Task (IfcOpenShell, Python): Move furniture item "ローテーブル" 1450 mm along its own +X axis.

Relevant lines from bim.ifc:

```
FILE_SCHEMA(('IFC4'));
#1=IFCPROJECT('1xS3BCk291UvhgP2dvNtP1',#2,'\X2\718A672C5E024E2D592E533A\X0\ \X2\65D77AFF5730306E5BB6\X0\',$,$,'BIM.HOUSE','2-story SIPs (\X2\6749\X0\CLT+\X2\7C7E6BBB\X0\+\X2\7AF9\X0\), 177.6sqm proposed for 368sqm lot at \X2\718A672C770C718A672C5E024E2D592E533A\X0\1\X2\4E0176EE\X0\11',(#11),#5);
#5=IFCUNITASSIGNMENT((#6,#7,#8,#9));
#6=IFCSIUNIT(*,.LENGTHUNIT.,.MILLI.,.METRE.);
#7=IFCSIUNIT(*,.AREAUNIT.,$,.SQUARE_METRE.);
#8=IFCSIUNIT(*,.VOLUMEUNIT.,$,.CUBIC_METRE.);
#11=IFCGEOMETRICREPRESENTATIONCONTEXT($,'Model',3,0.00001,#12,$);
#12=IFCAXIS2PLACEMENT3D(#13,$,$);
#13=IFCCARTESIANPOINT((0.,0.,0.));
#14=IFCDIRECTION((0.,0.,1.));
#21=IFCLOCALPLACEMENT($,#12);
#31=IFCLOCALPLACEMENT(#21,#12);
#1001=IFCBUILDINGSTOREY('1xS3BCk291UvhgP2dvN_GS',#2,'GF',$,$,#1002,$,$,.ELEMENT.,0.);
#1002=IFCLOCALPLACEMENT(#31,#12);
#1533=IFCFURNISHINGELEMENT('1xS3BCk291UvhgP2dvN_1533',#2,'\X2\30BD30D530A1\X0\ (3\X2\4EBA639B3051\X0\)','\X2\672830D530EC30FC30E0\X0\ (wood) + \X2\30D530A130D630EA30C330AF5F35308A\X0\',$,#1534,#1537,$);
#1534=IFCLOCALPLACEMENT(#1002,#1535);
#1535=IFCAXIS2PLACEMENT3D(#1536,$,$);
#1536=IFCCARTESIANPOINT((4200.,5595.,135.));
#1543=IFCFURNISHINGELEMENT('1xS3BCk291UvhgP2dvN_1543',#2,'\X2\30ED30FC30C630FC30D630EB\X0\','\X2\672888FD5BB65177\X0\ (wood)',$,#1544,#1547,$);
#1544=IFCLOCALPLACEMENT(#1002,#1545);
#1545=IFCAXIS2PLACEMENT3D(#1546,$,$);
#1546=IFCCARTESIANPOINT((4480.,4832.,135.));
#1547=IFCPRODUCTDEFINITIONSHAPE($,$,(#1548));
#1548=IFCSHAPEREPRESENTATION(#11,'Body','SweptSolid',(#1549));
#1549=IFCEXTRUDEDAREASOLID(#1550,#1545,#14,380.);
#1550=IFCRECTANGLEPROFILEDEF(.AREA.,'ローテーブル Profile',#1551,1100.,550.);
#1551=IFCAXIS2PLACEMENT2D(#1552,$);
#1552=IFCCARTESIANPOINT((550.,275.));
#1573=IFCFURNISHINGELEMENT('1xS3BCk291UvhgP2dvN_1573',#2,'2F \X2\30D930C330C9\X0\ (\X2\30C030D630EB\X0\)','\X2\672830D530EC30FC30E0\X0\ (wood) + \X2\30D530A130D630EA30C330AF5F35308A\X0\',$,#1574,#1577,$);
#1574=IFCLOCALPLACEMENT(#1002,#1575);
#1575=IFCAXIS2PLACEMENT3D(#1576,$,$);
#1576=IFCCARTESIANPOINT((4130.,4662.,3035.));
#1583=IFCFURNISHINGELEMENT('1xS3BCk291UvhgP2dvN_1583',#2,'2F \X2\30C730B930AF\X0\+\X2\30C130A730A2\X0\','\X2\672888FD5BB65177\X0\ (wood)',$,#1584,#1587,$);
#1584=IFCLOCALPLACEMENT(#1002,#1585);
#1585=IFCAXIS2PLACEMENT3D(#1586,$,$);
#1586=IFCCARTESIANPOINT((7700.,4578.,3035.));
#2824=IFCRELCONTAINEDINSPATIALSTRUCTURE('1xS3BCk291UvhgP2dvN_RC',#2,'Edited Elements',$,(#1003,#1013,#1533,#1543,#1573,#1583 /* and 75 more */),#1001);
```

```python
import ifcopenshell
import ifcopenshell.api.geometry
import ifcopenshell.util.placement
import ifcopenshell.util.unit

model = ifcopenshell.open("bim.ifc")
unit_scale = ifcopenshell.util.unit.calculate_unit_scale(model)

item = model.by_guid("1xS3BCk291UvhgP2dvN_1543")
matrix = ifcopenshell.util.placement.get_local_placement(item.ObjectPlacement)
matrix[:3, 3] += matrix[:3, 0] * 1.45 / unit_scale
ifcopenshell.api.geometry.edit_object_placement(model, product=item, matrix=matrix, is_si=False)

print(ifcopenshell.util.placement.get_local_placement(item.ObjectPlacement).round(3) + 0.0)

model.write("bim-out.ifc")
```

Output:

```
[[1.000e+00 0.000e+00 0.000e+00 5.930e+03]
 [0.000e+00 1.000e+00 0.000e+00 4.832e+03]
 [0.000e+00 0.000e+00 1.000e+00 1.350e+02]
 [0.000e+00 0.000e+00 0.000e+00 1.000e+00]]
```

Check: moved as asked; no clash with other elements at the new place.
